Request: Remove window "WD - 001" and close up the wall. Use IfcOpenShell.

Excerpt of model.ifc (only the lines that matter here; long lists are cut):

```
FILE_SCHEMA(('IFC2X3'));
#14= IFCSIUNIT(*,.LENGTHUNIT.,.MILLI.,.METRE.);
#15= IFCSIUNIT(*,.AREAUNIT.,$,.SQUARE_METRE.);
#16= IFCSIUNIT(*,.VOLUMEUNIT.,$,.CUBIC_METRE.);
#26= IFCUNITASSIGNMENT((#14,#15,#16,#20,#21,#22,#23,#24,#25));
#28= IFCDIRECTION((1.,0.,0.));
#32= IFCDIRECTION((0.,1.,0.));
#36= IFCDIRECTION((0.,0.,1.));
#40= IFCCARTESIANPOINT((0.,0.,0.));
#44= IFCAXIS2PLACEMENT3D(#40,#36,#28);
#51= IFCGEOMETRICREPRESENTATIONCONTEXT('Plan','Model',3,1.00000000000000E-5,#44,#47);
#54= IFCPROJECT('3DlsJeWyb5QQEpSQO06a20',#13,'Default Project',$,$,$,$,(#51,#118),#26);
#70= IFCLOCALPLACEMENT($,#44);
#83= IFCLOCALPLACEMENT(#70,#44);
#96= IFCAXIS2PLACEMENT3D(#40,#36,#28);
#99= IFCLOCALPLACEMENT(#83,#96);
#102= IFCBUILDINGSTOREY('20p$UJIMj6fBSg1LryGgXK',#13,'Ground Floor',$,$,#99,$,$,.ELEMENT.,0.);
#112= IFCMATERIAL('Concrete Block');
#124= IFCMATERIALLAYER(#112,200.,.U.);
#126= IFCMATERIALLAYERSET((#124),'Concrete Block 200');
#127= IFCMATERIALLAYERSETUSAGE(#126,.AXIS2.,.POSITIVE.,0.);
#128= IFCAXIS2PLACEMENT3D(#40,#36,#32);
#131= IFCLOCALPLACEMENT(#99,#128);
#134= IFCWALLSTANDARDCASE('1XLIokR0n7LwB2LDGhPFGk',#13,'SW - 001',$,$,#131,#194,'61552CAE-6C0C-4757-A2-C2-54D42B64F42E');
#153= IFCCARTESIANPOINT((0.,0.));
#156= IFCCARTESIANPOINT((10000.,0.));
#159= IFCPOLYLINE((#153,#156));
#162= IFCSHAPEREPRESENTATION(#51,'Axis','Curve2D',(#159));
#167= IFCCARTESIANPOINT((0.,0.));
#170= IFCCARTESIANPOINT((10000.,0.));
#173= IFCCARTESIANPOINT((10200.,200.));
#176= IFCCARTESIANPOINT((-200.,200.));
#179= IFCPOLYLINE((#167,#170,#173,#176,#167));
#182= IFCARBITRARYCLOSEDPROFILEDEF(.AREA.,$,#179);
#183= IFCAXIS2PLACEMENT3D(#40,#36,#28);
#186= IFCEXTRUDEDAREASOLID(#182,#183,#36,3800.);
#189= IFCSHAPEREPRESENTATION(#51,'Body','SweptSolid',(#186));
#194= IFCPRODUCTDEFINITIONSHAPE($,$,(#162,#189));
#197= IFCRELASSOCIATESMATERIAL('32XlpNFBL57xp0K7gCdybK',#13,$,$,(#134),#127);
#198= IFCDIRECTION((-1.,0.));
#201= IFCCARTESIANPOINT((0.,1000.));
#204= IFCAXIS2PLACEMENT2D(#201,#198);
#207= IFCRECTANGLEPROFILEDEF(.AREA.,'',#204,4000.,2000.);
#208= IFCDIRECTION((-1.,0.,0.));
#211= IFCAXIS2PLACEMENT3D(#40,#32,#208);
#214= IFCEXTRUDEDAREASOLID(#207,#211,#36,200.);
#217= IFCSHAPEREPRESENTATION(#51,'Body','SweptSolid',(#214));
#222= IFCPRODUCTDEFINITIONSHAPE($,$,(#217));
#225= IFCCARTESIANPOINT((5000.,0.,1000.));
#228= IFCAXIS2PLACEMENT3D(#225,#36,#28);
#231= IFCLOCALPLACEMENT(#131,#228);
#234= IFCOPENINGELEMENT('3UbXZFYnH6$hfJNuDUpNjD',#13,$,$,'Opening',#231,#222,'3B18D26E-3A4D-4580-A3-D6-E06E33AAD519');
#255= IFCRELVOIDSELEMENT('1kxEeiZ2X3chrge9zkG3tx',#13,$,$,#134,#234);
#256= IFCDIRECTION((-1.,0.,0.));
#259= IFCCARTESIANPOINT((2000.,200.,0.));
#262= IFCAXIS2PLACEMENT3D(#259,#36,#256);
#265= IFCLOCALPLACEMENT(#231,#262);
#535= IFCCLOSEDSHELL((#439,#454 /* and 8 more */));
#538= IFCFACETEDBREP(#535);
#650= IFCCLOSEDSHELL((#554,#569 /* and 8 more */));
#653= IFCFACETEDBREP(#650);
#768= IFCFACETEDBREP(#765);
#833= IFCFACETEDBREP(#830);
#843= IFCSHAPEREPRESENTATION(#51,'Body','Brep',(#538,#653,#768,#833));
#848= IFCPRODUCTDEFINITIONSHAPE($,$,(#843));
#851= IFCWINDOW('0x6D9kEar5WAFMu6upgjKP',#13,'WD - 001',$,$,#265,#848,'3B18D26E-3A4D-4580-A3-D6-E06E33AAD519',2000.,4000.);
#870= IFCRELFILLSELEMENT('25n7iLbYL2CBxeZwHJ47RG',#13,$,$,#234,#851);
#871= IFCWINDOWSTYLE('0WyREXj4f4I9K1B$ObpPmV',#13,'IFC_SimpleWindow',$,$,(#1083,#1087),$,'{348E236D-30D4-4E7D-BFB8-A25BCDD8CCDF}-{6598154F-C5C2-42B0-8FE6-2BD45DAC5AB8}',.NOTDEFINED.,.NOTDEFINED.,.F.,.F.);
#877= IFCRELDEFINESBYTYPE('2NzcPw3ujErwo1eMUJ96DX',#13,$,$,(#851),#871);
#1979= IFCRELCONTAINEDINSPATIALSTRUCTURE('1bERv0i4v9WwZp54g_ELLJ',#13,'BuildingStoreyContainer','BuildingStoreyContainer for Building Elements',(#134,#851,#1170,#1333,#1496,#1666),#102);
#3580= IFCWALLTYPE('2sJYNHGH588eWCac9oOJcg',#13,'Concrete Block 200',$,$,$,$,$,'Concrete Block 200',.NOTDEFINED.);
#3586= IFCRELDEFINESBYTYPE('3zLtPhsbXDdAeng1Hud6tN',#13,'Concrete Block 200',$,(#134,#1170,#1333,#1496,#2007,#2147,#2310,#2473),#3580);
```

```python
import ifcopenshell
import ifcopenshell.api.feature
import ifcopenshell.api.root
import ifcopenshell.geom
import ifcopenshell.util.shape

model = ifcopenshell.open("model.ifc")
settings = ifcopenshell.geom.settings()


def volume(element):
    """Net volume in cubic metres, openings subtracted."""
    shape = ifcopenshell.geom.create_shape(settings, element)
    return ifcopenshell.util.shape.get_volume(shape.geometry)


window = model.by_guid("0x6D9kEar5WAFMu6upgjKP")
opening = window.FillsVoids[0].RelatingOpeningElement
wall = opening.VoidsElements[0].RelatingBuildingElement
before = volume(wall)

ifcopenshell.api.root.remove_product(model, product=window)
ifcopenshell.api.feature.remove_feature(model, feature=opening)

after = volume(wall)

print(f"wall volume {before:.3f} -> {after:.3f} m3")

model.write("model_v2.ifc")
```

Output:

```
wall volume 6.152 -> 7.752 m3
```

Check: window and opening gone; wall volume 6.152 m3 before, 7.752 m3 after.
